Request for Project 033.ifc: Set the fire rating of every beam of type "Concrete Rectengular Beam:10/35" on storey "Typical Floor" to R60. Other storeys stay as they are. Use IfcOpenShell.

First a look at what the model holds.

```python
import ifcopenshell
import ifcopenshell.util.element

model = ifcopenshell.open("Project 033.ifc")
print(model.schema)
storey = next(s for s in model.by_type("IfcBuildingStorey") if s.Name == "Typical Floor")
beams = [e for e in ifcopenshell.util.element.get_decomposition(storey) if e.is_a("IfcBeam")]
seen = {}
for e in beams:
    element_type = ifcopenshell.util.element.get_type(e)
    key = (element_type.Name if element_type != e and element_type else None, ifcopenshell.util.element.get_pset(e, "Pset_BeamCommon", "FireRating"))
    seen[key] = seen.get(key, 0) + 1
for (name, value), count in sorted(seen.items(), key=str):
    print(count, "x", name, "|", value)
```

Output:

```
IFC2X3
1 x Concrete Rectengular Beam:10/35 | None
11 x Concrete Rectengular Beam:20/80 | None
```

```python
import ifcopenshell
import ifcopenshell.api.pset
import ifcopenshell.util.element

model = ifcopenshell.open("Project 033.ifc")

storey = next(s for s in model.by_type("IfcBuildingStorey") if s.Name == "Typical Floor")
beams = [e for e in ifcopenshell.util.element.get_decomposition(storey) if e.is_a("IfcBeam")]

count = 0
for e in beams:
    element_type = ifcopenshell.util.element.get_type(e)
    if element_type in (None, e) or element_type.Name != "Concrete Rectengular Beam:10/35":
        continue
    # add_pset returns the element's existing set when there is one.
    pset = ifcopenshell.api.pset.add_pset(model, product=e, name="Pset_BeamCommon")
    ifcopenshell.api.pset.edit_pset(model, pset=pset, properties={"FireRating": "R60"})
    count += 1

print(count, "beams updated")

model.write("Project 033_updated.ifc")
```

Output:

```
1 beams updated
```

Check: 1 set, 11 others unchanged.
